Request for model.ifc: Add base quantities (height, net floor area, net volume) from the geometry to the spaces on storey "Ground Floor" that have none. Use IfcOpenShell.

First a look at what the model holds.

```python
import ifcopenshell
import ifcopenshell.util.element
import ifcopenshell.util.unit

model = ifcopenshell.open("model.ifc")
print(model.schema)
for unit_type in ("LENGTHUNIT", "AREAUNIT", "VOLUMEUNIT"):
    print(unit_type, ifcopenshell.util.unit.calculate_unit_scale(model, unit_type))
storey = next(s for s in model.by_type("IfcBuildingStorey") if s.Name == "Ground Floor")
spaces = [e for e in ifcopenshell.util.element.get_decomposition(storey) if e.is_a("IfcSpace")]
for e in sorted(spaces, key=lambda e: e.id()):
    print(e.id(), e.is_a(), e.Name, list(ifcopenshell.util.element.get_psets(e, qtos_only=True)), sep=" | ")
```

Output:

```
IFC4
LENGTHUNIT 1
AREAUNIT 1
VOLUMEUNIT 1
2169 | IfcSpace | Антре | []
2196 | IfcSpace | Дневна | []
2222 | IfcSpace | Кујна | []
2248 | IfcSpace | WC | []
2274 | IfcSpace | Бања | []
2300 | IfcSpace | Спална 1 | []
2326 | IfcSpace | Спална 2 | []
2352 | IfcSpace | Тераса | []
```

```python
import ifcopenshell
import ifcopenshell.api.pset
import ifcopenshell.geom
import ifcopenshell.util.element
import ifcopenshell.util.shape
import ifcopenshell.util.unit

model = ifcopenshell.open("model.ifc")
unit_scale = ifcopenshell.util.unit.calculate_unit_scale(model)
area_scale = ifcopenshell.util.unit.calculate_unit_scale(model, "AREAUNIT")
volume_scale = ifcopenshell.util.unit.calculate_unit_scale(model, "VOLUMEUNIT")
settings = ifcopenshell.geom.settings()

storey = next(s for s in model.by_type("IfcBuildingStorey") if s.Name == "Ground Floor")
spaces = [e for e in ifcopenshell.util.element.get_decomposition(storey) if e.is_a("IfcSpace")]

for e in sorted(spaces, key=lambda e: e.id()):
    if ifcopenshell.util.element.get_psets(e, qtos_only=True, should_inherit=False):
        continue
    # Geometry comes back in metres, in the element's own axes.
    shape = ifcopenshell.geom.create_shape(settings, e)
    values = {
        "Height": ifcopenshell.util.shape.get_z(shape.geometry) / unit_scale,
        "NetFloorArea": ifcopenshell.util.shape.get_footprint_area(shape.geometry) / area_scale,
        "NetVolume": ifcopenshell.util.shape.get_volume(shape.geometry) / volume_scale,
    }
    qto = ifcopenshell.api.pset.add_qto(model, product=e, name="Qto_SpaceBaseQuantities")
    ifcopenshell.api.pset.edit_qto(model, qto=qto, properties=values)
    print(e.id(), {k: round(v, 3) for k, v in values.items()})

model.write("model_edited.ifc")
```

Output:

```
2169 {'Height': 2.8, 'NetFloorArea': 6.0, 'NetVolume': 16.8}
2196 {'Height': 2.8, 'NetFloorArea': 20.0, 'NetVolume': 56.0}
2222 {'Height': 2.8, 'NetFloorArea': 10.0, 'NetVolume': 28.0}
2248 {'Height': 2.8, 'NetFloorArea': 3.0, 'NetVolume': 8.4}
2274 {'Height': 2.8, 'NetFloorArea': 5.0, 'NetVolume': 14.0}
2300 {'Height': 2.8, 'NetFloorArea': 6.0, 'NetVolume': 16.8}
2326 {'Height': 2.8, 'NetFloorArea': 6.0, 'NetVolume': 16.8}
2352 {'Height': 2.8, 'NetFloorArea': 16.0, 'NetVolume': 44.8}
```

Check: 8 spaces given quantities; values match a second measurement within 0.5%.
